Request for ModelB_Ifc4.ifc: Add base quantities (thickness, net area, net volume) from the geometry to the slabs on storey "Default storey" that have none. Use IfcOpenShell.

First a look at what the model holds.

```python
import ifcopenshell
import ifcopenshell.util.element
import ifcopenshell.util.unit

model = ifcopenshell.open("ModelB_Ifc4.ifc")
print(model.schema)
for unit_type in ("LENGTHUNIT", "AREAUNIT", "VOLUMEUNIT"):
    print(unit_type, ifcopenshell.util.unit.calculate_unit_scale(model, unit_type))
storey = next(s for s in model.by_type("IfcBuildingStorey") if s.Name == "Default storey")
slabs = [e for e in ifcopenshell.util.element.get_decomposition(storey) if e.is_a("IfcSlab")]
for e in sorted(slabs, key=lambda e: e.id()):
    print(e.id(), e.is_a(), e.Name, list(ifcopenshell.util.element.get_psets(e, qtos_only=True)), sep=" | ")
```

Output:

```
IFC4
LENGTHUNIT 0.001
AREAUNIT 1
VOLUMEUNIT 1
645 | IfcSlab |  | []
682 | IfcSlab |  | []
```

```python
import ifcopenshell
import ifcopenshell.api.pset
import ifcopenshell.geom
import ifcopenshell.util.element
import ifcopenshell.util.shape
import ifcopenshell.util.unit

model = ifcopenshell.open("ModelB_Ifc4.ifc")
unit_scale = ifcopenshell.util.unit.calculate_unit_scale(model)
area_scale = ifcopenshell.util.unit.calculate_unit_scale(model, "AREAUNIT")
volume_scale = ifcopenshell.util.unit.calculate_unit_scale(model, "VOLUMEUNIT")
settings = ifcopenshell.geom.settings()

storey = next(s for s in model.by_type("IfcBuildingStorey") if s.Name == "Default storey")
slabs = [e for e in ifcopenshell.util.element.get_decomposition(storey) if e.is_a("IfcSlab")]

for e in sorted(slabs, key=lambda e: e.id()):
    if ifcopenshell.util.element.get_psets(e, qtos_only=True, should_inherit=False):
        continue
    # Geometry comes back in metres, in the element's own axes.
    shape = ifcopenshell.geom.create_shape(settings, e)
    values = {
        "Width": ifcopenshell.util.shape.get_z(shape.geometry) / unit_scale,
        "NetArea": ifcopenshell.util.shape.get_footprint_area(shape.geometry) / area_scale,
        "NetVolume": ifcopenshell.util.shape.get_volume(shape.geometry) / volume_scale,
    }
    qto = ifcopenshell.api.pset.add_qto(model, product=e, name="Qto_SlabBaseQuantities")
    ifcopenshell.api.pset.edit_qto(model, qto=qto, properties=values)
    print(e.id(), {k: round(v, 3) for k, v in values.items()})

model.write("ModelB_Ifc4-out.ifc")
```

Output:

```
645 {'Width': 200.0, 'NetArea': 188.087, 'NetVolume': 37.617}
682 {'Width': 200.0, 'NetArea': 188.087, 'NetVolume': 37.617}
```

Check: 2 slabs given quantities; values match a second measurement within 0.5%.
